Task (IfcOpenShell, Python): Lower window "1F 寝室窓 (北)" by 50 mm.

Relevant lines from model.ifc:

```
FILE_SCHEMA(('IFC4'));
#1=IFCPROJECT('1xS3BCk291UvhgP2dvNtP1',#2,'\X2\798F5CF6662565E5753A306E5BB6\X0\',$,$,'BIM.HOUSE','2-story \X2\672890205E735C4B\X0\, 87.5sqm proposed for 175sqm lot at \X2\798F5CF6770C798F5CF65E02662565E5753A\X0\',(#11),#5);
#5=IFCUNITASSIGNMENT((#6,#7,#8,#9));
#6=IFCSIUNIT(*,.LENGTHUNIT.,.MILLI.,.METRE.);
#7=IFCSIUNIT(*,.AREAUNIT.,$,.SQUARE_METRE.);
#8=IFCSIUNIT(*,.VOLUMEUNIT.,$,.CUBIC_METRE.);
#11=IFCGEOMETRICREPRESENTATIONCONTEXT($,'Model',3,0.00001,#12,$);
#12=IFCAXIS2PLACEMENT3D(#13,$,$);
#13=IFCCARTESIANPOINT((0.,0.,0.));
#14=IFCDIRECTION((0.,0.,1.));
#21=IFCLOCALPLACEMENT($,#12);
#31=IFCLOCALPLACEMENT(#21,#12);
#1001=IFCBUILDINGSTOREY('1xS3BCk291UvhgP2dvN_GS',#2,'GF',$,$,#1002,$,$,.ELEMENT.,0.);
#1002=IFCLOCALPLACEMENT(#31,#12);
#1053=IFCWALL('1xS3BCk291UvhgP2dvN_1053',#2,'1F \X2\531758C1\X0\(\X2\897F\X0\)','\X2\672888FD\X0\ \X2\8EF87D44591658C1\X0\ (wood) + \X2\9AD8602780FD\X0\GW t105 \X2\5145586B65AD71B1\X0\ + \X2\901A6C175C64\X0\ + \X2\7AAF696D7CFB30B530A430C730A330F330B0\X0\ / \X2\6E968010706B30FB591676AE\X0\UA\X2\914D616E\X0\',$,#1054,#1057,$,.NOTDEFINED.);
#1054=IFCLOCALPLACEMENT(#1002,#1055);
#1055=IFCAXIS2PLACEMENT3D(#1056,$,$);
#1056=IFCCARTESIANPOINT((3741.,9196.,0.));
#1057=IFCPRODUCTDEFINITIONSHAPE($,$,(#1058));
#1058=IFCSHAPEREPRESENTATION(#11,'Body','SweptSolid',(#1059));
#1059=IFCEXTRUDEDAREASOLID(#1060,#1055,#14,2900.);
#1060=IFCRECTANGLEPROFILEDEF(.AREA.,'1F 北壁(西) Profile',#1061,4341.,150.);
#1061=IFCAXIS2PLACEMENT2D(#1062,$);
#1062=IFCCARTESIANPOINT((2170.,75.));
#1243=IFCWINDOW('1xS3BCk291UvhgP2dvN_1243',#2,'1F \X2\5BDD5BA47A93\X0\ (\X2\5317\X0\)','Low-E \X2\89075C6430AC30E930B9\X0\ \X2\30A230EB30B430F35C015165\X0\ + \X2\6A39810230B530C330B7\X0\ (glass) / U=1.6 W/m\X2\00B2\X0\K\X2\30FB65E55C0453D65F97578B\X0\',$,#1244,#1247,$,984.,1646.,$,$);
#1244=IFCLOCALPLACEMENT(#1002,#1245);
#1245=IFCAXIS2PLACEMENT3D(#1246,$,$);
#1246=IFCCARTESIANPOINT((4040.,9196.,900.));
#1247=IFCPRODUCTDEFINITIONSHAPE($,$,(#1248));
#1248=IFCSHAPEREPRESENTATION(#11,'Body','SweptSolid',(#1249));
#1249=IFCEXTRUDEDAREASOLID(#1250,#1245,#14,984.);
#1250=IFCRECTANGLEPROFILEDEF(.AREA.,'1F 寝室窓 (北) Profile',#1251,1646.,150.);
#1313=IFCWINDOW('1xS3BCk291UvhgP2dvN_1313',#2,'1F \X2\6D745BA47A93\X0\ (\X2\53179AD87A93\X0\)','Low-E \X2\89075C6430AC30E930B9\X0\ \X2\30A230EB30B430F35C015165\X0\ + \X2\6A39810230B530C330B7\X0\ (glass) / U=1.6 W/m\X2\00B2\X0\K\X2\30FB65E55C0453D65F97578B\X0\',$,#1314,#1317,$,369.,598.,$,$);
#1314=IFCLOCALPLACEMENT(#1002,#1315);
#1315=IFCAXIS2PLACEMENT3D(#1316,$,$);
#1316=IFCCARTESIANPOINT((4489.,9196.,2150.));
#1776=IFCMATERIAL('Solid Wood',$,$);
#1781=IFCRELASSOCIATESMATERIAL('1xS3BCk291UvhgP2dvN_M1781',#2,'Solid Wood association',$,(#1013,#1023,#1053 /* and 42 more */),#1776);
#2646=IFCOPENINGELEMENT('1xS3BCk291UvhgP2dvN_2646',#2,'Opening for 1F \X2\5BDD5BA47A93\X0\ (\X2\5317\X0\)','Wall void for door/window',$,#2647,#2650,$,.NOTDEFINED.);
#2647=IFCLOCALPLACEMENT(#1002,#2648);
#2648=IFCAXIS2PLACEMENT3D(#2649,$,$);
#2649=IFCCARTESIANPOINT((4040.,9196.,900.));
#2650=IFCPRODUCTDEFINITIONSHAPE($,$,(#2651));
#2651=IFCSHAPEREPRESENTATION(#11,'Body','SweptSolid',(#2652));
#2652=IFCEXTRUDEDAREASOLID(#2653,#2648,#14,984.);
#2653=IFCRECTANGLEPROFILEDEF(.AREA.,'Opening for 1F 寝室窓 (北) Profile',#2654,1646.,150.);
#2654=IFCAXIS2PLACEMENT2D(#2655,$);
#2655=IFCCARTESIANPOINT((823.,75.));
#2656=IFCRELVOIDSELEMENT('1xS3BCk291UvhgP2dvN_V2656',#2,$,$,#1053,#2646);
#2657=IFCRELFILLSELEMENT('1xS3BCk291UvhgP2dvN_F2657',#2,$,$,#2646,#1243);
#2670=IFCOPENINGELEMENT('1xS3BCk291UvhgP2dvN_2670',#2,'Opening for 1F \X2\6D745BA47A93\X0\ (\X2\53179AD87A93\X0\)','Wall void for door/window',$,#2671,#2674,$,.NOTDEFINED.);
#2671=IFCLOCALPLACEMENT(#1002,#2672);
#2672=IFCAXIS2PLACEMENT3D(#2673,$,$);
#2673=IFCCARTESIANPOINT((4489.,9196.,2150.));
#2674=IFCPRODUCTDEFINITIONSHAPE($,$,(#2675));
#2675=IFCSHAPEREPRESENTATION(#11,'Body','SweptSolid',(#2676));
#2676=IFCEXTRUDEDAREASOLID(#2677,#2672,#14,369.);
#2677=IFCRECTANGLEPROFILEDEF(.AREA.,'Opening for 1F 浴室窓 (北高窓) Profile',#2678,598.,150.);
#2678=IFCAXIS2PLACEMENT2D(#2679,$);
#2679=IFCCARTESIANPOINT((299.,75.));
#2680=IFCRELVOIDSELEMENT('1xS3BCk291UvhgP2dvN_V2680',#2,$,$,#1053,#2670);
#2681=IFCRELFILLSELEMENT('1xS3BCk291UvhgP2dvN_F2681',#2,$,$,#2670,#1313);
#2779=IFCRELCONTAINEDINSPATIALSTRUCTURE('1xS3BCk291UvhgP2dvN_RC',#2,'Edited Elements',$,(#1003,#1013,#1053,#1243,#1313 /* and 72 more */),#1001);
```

```python
import numpy as np
import ifcopenshell
import ifcopenshell.api.geometry
import ifcopenshell.util.placement
import ifcopenshell.util.unit

model = ifcopenshell.open("model.ifc")
unit_scale = ifcopenshell.util.unit.calculate_unit_scale(model)

window = model.by_guid("1xS3BCk291UvhgP2dvN_1243")
opening = window.FillsVoids[0].RelatingOpeningElement
dz = -0.05 / unit_scale

shift = np.array([0.0, 0.0, dz])
# The window is not placed relative to its opening, so move both.
for product in (opening, window):
    matrix = ifcopenshell.util.placement.get_local_placement(product.ObjectPlacement)
    matrix[:3, 3] += shift
    ifcopenshell.api.geometry.edit_object_placement(model, product=product, matrix=matrix, is_si=False)

print(f"moved by {dz * unit_scale:+.3f} m")

model.write("model_rev.ifc")
```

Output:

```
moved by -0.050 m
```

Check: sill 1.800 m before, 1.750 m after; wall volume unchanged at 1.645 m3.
